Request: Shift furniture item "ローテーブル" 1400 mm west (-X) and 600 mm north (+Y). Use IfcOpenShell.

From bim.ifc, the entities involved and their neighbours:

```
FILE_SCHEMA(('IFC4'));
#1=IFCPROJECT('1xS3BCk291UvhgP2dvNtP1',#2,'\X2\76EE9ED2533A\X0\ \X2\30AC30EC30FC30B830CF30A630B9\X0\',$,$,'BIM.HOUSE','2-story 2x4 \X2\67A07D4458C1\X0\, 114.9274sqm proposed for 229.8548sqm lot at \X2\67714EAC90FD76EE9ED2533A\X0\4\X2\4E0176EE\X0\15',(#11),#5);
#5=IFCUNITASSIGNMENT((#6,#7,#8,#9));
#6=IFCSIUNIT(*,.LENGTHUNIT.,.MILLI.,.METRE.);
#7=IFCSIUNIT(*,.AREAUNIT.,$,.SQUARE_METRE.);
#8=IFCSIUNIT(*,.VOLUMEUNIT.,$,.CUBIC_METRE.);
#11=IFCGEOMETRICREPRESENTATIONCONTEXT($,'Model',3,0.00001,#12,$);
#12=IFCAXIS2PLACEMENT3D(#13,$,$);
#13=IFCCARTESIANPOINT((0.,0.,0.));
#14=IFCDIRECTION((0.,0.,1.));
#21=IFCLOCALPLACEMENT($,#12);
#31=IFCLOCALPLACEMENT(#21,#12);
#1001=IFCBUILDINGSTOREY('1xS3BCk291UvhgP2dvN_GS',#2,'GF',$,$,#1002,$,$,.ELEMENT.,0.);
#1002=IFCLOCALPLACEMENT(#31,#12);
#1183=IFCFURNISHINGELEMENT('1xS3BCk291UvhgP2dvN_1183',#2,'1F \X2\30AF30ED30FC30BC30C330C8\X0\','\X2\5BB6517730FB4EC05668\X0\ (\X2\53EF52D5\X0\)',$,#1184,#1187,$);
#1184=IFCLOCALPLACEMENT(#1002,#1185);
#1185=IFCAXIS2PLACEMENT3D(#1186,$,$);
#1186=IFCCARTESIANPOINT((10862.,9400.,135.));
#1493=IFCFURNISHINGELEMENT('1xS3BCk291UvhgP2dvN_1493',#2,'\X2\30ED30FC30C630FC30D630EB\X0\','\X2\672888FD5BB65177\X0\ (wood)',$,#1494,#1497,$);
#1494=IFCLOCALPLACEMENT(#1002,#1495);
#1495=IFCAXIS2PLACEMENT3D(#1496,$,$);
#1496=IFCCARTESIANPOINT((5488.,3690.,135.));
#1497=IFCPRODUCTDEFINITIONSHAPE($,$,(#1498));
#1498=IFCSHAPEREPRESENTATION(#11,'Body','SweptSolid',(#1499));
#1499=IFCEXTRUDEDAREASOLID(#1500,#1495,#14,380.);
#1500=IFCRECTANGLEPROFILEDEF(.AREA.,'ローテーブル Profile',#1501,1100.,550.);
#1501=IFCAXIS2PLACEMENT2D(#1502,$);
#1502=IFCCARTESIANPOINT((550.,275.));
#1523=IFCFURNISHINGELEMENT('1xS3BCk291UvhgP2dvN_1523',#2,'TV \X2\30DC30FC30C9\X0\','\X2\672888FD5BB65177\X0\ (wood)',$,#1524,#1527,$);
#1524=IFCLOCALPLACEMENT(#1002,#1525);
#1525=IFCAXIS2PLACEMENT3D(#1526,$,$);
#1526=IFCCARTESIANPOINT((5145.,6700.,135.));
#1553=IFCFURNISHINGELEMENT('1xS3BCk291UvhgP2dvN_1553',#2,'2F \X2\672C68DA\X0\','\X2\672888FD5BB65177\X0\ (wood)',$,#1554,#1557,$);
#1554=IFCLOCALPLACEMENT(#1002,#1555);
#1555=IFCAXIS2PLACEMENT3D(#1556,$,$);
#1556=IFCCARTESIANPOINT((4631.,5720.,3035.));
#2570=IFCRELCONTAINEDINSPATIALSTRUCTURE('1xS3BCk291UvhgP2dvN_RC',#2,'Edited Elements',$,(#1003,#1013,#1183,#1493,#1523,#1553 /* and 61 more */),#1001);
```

```python
import ifcopenshell
import ifcopenshell.api.geometry
import ifcopenshell.util.placement
import ifcopenshell.util.unit

model = ifcopenshell.open("bim.ifc")
unit_scale = ifcopenshell.util.unit.calculate_unit_scale(model)

item = model.by_guid("1xS3BCk291UvhgP2dvN_1493")
matrix = ifcopenshell.util.placement.get_local_placement(item.ObjectPlacement)
matrix[0, 3] -= 1.4 / unit_scale
matrix[1, 3] += 0.6 / unit_scale
ifcopenshell.api.geometry.edit_object_placement(model, product=item, matrix=matrix, is_si=False)

print(ifcopenshell.util.placement.get_local_placement(item.ObjectPlacement).round(3) + 0.0)

model.write("bim_edited.ifc")
```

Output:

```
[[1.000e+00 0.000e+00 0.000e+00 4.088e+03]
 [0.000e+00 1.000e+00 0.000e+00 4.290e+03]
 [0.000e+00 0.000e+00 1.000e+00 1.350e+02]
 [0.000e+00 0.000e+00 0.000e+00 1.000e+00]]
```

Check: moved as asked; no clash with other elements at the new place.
